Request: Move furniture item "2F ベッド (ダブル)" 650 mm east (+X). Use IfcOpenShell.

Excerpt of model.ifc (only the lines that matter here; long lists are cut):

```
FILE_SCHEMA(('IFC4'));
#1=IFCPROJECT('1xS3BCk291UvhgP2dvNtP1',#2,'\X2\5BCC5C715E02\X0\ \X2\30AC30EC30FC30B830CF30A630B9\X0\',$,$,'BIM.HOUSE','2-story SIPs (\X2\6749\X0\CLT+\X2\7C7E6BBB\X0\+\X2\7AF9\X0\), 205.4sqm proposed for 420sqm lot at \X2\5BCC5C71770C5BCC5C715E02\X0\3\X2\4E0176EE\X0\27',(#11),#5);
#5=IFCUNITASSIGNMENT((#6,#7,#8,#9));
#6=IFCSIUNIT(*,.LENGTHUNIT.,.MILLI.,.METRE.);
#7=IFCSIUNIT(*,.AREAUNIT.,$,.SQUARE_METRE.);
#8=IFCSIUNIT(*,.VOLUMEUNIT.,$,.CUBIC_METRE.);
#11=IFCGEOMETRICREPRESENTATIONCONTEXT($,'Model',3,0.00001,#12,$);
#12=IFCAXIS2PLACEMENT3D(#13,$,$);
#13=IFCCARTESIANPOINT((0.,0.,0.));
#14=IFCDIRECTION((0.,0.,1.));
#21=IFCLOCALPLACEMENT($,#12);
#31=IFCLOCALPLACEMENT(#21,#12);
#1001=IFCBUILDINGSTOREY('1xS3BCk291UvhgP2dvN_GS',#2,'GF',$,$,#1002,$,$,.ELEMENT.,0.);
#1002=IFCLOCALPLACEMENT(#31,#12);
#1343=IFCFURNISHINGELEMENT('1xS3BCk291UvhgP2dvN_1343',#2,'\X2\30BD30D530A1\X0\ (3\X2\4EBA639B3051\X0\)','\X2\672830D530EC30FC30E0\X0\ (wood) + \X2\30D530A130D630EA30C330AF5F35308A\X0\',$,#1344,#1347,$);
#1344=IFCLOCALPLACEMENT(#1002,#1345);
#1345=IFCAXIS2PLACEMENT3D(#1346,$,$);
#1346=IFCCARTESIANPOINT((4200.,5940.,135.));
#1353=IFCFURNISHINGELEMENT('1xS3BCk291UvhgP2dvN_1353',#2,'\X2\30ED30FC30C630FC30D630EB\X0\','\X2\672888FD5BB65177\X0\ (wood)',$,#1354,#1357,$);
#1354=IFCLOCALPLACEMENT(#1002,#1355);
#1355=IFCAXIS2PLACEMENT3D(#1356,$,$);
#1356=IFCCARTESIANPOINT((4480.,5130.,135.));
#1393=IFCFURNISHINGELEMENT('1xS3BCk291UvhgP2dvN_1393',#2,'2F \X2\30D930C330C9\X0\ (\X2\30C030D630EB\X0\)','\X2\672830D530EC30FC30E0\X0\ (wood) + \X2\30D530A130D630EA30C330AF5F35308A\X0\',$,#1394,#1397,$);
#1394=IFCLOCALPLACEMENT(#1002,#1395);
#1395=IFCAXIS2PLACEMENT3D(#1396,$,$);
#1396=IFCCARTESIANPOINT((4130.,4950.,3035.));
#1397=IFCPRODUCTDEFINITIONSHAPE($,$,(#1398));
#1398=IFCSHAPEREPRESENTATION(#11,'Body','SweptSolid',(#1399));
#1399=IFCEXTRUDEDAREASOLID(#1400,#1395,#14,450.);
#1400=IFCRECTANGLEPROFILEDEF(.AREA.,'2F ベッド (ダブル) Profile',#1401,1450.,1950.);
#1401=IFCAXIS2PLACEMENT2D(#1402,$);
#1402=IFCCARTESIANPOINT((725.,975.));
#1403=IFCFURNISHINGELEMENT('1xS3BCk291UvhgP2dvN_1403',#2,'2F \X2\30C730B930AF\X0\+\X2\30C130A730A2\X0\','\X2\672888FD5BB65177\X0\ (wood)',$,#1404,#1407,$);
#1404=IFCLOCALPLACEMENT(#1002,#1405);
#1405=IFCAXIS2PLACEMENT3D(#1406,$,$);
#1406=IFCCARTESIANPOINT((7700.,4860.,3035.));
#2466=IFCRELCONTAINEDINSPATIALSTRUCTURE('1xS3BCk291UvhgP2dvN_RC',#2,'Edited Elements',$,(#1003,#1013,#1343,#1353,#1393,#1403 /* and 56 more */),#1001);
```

```python
import ifcopenshell
import ifcopenshell.api.geometry
import ifcopenshell.util.placement
import ifcopenshell.util.unit

model = ifcopenshell.open("model.ifc")
unit_scale = ifcopenshell.util.unit.calculate_unit_scale(model)

item = model.by_id(1393)
matrix = ifcopenshell.util.placement.get_local_placement(item.ObjectPlacement)
matrix[0, 3] += 0.65 / unit_scale
ifcopenshell.api.geometry.edit_object_placement(model, product=item, matrix=matrix, is_si=False)

print(ifcopenshell.util.placement.get_local_placement(item.ObjectPlacement).round(3) + 0.0)

model.write("model_rev.ifc")
```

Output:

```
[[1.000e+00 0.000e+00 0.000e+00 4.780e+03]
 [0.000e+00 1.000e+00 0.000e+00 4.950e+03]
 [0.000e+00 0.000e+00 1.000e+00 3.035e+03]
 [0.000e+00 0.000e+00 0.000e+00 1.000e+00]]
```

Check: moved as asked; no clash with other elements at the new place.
